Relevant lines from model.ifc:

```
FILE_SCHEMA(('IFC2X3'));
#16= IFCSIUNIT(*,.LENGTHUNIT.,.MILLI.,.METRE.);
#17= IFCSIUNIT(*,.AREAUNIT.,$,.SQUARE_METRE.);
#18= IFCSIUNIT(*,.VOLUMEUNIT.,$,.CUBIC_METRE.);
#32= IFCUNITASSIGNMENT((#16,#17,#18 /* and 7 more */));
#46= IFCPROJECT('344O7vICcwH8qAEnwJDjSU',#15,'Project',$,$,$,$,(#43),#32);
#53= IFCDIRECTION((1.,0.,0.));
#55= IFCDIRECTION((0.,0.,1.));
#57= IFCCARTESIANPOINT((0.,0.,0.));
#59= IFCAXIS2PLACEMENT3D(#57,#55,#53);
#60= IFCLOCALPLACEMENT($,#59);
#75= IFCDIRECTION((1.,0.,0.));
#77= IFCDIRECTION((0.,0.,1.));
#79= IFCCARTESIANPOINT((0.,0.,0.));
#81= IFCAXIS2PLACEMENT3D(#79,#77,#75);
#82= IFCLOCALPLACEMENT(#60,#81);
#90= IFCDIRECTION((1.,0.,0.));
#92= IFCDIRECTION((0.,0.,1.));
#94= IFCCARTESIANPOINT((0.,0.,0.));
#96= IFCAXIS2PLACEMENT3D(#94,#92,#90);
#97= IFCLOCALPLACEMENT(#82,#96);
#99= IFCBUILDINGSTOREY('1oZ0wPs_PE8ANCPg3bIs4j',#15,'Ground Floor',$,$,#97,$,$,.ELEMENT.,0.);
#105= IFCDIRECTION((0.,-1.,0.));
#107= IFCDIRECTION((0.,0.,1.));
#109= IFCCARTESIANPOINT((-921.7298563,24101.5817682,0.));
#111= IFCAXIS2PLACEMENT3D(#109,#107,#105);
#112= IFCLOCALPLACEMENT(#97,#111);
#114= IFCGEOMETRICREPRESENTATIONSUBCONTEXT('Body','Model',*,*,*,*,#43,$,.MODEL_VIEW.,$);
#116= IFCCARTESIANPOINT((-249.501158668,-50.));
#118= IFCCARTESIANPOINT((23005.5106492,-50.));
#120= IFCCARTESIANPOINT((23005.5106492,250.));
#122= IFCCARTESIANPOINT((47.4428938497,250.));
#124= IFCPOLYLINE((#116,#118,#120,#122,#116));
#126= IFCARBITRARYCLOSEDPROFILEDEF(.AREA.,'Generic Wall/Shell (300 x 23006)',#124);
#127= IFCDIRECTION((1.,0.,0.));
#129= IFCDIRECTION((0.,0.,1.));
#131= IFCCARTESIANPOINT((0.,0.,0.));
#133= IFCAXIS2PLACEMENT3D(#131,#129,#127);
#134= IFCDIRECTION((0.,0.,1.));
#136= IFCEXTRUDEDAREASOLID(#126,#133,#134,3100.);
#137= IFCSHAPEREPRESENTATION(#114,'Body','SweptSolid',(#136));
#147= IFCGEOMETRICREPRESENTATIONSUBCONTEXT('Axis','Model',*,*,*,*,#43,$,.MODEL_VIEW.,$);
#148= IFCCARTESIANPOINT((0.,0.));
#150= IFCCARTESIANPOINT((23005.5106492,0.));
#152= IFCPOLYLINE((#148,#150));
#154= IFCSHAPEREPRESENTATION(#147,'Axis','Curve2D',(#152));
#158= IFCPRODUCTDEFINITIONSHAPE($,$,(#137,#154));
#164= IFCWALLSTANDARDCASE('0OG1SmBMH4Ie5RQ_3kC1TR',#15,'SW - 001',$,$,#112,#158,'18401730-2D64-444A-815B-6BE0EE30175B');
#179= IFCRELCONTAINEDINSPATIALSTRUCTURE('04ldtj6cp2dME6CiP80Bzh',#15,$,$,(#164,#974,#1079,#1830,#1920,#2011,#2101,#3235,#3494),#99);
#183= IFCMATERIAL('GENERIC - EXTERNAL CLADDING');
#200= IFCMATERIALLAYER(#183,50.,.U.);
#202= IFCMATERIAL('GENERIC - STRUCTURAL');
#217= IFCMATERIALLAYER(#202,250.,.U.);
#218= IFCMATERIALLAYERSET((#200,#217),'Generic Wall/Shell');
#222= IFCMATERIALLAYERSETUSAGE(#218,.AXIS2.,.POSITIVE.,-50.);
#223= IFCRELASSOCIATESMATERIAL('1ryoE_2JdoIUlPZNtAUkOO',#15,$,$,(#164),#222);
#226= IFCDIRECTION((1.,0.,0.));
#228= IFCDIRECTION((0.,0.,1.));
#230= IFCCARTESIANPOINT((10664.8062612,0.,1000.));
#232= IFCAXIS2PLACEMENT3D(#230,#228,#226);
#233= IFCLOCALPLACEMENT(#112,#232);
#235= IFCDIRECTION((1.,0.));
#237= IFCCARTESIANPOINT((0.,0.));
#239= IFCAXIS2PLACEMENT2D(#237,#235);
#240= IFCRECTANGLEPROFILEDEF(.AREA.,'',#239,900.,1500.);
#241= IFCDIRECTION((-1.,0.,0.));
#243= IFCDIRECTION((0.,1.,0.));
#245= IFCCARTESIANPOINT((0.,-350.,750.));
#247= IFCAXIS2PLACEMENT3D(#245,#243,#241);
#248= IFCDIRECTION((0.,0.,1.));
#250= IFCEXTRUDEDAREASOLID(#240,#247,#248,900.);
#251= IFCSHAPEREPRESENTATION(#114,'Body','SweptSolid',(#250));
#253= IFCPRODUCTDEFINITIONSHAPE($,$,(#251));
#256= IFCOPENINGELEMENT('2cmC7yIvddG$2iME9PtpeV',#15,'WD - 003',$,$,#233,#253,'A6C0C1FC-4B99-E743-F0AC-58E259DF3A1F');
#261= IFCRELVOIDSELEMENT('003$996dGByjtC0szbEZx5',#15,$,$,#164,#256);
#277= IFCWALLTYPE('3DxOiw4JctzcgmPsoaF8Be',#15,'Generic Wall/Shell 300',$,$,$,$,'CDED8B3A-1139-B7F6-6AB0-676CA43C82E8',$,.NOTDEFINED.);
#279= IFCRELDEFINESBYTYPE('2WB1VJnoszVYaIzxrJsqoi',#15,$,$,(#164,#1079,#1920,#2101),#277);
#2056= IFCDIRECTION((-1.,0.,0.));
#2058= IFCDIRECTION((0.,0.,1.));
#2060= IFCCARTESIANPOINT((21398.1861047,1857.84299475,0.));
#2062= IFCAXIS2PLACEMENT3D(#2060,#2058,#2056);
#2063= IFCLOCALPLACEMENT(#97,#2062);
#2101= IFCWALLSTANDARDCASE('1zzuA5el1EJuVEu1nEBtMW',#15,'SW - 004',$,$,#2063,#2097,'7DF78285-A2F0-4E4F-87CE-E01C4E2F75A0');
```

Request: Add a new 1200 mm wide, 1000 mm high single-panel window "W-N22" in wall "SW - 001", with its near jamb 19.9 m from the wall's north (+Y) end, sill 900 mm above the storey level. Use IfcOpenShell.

```python
import numpy as np
import ifcopenshell
import ifcopenshell.api.feature
import ifcopenshell.api.geometry
import ifcopenshell.api.root
import ifcopenshell.api.spatial
import ifcopenshell.api.type
import ifcopenshell.geom
import ifcopenshell.util.element
import ifcopenshell.util.placement
import ifcopenshell.util.representation
import ifcopenshell.util.shape
import ifcopenshell.util.unit

model = ifcopenshell.open("model.ifc")
unit_scale = ifcopenshell.util.unit.calculate_unit_scale(model)
settings = ifcopenshell.geom.settings()


def volume(element):
    """Net volume in cubic metres, openings subtracted."""
    shape = ifcopenshell.geom.create_shape(settings, element)
    return ifcopenshell.util.shape.get_volume(shape.geometry)


wall = model.by_guid("0OG1SmBMH4Ie5RQ_3kC1TR")
storey = ifcopenshell.util.element.get_container(wall, ifc_class="IfcBuildingStorey")
context = ifcopenshell.util.representation.get_context(model, "Model", "Body", "MODEL_VIEW")
before = volume(wall)

width, height, from_end, sill = 1.2, 1, 19.9, 0.9  # metres

# The wall runs along its own X axis, and the end named is its -X end.
wall_shape = ifcopenshell.geom.create_shape(settings, wall)
x, y, z = ifcopenshell.util.shape.get_vertices(wall_shape.geometry).T
start = x.min() + from_end
face, thickness = float(y.min()), float(y.max() - y.min())
wall_matrix = ifcopenshell.util.placement.get_local_placement(wall.ObjectPlacement)
level = ifcopenshell.util.placement.get_local_placement(storey.ObjectPlacement)[2, 3]


def in_wall(x, y):
    """Placement at x, y metres in the wall's axes, at sill height."""
    matrix = wall_matrix.copy()
    matrix[:, 3] = wall_matrix @ np.array([x / unit_scale, y / unit_scale, 0.0, 1.0])
    matrix[2, 3] = level + sill / unit_scale
    return matrix


# Opening: a box that overshoots both wall faces by 50 mm.
opening = ifcopenshell.api.root.create_entity(model, ifc_class="IfcOpeningElement")
box = ifcopenshell.api.geometry.add_wall_representation(
    model, context=context, length=width, height=height, thickness=thickness + 0.1
)
ifcopenshell.api.geometry.assign_representation(model, product=opening, representation=box)
ifcopenshell.api.geometry.edit_object_placement(model, product=opening, matrix=in_wall(start, face - 0.05), is_si=False)
ifcopenshell.api.feature.add_feature(model, feature=opening, element=wall)

window = ifcopenshell.api.root.create_entity(model, ifc_class="IfcWindow", name="W-N22")
window.OverallWidth, window.OverallHeight = width / unit_scale, height / unit_scale
body = ifcopenshell.api.geometry.add_window_representation(
    model,
    context=context,
    overall_width=window.OverallWidth,
    overall_height=window.OverallHeight,
    partition_type="SINGLE_PANEL",
)
ifcopenshell.api.geometry.assign_representation(model, product=window, representation=body)
ifcopenshell.api.spatial.assign_container(model, products=[window], relating_structure=storey)
fills = ifcopenshell.api.feature.add_filling(model, opening=opening, element=window)
fills.OwnerHistory = window.OwnerHistory  # required in IFC2X3

# IFC2X3 keeps the operation on the window style.
style = ifcopenshell.api.root.create_entity(model, ifc_class="IfcWindowStyle", name="W-N22")
style.OperationType, style.ConstructionType = "SINGLE_PANEL", "NOTDEFINED"
style.ParameterTakesPrecedence = style.Sizeable = False
ifcopenshell.api.type.assign_type(model, related_objects=[window], relating_type=style)

# Centre the window in the wall's thickness.
ifcopenshell.api.geometry.edit_object_placement(model, product=window, matrix=in_wall(start, face), is_si=False)
window_shape = ifcopenshell.geom.create_shape(settings, window)
depth = ifcopenshell.util.shape.get_vertices(window_shape.geometry)[:, 1]
offset = face + thickness / 2 - (depth.min() + depth.max()) / 2
ifcopenshell.api.geometry.edit_object_placement(model, product=window, matrix=in_wall(start, offset), is_si=False)

after = volume(wall)

print(f"wall volume {before:.3f} -> {after:.3f} m3")

model.write("model_rev.ifc")
```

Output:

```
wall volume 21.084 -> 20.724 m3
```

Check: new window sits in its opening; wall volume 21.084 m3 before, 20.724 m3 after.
